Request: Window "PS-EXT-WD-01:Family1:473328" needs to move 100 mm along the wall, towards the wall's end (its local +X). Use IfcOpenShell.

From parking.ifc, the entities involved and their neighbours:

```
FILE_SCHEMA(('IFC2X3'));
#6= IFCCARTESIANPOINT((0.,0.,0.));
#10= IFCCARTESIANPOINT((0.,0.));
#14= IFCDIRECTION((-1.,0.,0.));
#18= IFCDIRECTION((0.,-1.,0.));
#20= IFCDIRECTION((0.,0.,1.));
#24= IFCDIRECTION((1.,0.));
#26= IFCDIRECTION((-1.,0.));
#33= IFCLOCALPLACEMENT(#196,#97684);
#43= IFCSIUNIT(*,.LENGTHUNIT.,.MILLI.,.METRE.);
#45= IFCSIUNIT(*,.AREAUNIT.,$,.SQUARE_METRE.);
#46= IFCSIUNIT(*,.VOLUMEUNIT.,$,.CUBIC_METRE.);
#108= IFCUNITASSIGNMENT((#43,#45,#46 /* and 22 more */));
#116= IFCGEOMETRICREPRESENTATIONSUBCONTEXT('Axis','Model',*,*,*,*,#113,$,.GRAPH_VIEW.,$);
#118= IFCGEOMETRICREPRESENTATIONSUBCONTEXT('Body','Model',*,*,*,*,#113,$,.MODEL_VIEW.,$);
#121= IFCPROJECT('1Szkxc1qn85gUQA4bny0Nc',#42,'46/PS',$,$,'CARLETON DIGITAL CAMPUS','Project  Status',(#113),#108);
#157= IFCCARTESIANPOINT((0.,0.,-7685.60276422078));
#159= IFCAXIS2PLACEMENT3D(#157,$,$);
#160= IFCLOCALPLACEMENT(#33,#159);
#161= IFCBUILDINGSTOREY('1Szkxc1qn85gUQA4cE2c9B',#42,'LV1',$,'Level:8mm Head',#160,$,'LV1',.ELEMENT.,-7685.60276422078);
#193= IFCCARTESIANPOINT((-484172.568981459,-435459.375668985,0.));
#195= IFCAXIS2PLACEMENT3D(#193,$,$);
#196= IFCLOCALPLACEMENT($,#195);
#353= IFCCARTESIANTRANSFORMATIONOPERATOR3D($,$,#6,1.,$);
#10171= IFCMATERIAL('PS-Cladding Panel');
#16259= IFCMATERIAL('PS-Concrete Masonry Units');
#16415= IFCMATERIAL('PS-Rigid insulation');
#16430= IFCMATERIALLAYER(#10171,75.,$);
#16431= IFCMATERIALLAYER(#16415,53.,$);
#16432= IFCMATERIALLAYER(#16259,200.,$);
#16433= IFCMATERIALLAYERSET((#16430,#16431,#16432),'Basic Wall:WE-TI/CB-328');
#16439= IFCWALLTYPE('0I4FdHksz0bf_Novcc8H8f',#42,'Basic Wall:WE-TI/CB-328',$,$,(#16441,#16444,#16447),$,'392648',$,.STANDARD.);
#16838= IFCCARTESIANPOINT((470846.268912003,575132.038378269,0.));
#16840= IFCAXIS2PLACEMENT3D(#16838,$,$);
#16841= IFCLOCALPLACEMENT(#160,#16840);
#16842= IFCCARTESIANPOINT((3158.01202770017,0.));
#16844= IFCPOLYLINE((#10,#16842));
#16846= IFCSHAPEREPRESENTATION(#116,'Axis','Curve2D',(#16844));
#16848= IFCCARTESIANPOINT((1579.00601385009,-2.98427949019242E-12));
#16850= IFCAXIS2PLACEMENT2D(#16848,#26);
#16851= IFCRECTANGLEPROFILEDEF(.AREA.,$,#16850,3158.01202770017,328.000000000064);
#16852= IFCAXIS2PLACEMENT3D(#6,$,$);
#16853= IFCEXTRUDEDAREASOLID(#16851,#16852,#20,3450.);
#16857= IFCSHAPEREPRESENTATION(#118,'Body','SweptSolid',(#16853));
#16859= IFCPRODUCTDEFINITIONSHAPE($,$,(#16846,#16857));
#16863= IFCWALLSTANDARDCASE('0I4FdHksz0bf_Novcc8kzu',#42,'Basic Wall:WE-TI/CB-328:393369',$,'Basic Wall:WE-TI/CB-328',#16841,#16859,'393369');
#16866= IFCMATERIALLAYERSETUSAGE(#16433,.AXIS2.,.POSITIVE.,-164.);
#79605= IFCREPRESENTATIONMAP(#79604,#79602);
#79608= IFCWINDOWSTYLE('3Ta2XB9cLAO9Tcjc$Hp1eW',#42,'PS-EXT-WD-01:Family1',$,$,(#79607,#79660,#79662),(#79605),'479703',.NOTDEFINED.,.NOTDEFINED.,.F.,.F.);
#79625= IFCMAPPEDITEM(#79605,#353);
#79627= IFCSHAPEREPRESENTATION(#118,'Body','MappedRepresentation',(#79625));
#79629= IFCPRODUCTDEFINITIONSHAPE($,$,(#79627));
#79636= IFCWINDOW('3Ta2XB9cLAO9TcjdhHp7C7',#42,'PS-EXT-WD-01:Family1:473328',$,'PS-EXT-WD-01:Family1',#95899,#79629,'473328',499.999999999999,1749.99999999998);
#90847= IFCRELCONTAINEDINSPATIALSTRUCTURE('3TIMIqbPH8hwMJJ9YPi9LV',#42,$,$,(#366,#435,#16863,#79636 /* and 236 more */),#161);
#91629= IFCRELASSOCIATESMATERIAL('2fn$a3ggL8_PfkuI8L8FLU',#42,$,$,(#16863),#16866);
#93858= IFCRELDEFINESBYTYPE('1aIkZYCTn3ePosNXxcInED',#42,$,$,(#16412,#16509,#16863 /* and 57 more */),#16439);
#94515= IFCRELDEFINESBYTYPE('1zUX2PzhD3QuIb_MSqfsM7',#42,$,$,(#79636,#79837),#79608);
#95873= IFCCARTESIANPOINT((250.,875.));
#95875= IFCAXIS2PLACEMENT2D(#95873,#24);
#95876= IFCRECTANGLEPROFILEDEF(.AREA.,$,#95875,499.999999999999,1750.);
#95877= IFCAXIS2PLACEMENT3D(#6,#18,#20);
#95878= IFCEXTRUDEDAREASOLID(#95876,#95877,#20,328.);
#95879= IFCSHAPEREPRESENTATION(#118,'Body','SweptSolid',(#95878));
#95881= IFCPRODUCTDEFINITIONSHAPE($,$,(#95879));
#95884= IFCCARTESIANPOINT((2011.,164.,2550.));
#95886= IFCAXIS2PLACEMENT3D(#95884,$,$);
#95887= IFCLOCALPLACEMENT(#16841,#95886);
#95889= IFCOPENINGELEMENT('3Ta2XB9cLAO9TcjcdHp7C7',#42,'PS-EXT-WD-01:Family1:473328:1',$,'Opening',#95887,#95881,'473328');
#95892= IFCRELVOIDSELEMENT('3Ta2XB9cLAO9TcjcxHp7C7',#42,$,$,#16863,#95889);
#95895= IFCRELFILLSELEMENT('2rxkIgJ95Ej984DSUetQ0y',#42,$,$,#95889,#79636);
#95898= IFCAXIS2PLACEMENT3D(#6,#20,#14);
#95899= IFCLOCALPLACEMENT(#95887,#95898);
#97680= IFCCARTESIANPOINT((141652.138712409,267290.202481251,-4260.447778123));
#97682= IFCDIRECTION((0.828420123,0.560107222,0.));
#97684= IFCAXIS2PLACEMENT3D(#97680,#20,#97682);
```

```python
import ifcopenshell
import ifcopenshell.api.geometry
import ifcopenshell.util.placement

model = ifcopenshell.open("parking.ifc")

window = model.by_guid("3Ta2XB9cLAO9TcjdhHp7C7")
opening = window.FillsVoids[0].RelatingOpeningElement
wall = opening.VoidsElements[0].RelatingBuildingElement

wall_matrix = ifcopenshell.util.placement.get_local_placement(wall.ObjectPlacement)
shift = wall_matrix[:3, 0] * 100.0
before = ifcopenshell.util.placement.get_local_placement(window.ObjectPlacement)[:3, 3].copy()

# The window is placed relative to its opening, so it follows when the opening moves.
matrix = ifcopenshell.util.placement.get_local_placement(opening.ObjectPlacement)
matrix[:3, 3] += shift
ifcopenshell.api.geometry.edit_object_placement(
    model, product=opening, matrix=matrix, is_si=False, should_transform_children=True
)

after = ifcopenshell.util.placement.get_local_placement(window.ObjectPlacement)[:3, 3]
print("window moved by", (after - before).round(3) + 0.0)

model.write("parking_v2.ifc")
```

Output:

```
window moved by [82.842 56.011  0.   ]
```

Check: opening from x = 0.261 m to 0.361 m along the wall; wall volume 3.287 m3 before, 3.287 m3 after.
